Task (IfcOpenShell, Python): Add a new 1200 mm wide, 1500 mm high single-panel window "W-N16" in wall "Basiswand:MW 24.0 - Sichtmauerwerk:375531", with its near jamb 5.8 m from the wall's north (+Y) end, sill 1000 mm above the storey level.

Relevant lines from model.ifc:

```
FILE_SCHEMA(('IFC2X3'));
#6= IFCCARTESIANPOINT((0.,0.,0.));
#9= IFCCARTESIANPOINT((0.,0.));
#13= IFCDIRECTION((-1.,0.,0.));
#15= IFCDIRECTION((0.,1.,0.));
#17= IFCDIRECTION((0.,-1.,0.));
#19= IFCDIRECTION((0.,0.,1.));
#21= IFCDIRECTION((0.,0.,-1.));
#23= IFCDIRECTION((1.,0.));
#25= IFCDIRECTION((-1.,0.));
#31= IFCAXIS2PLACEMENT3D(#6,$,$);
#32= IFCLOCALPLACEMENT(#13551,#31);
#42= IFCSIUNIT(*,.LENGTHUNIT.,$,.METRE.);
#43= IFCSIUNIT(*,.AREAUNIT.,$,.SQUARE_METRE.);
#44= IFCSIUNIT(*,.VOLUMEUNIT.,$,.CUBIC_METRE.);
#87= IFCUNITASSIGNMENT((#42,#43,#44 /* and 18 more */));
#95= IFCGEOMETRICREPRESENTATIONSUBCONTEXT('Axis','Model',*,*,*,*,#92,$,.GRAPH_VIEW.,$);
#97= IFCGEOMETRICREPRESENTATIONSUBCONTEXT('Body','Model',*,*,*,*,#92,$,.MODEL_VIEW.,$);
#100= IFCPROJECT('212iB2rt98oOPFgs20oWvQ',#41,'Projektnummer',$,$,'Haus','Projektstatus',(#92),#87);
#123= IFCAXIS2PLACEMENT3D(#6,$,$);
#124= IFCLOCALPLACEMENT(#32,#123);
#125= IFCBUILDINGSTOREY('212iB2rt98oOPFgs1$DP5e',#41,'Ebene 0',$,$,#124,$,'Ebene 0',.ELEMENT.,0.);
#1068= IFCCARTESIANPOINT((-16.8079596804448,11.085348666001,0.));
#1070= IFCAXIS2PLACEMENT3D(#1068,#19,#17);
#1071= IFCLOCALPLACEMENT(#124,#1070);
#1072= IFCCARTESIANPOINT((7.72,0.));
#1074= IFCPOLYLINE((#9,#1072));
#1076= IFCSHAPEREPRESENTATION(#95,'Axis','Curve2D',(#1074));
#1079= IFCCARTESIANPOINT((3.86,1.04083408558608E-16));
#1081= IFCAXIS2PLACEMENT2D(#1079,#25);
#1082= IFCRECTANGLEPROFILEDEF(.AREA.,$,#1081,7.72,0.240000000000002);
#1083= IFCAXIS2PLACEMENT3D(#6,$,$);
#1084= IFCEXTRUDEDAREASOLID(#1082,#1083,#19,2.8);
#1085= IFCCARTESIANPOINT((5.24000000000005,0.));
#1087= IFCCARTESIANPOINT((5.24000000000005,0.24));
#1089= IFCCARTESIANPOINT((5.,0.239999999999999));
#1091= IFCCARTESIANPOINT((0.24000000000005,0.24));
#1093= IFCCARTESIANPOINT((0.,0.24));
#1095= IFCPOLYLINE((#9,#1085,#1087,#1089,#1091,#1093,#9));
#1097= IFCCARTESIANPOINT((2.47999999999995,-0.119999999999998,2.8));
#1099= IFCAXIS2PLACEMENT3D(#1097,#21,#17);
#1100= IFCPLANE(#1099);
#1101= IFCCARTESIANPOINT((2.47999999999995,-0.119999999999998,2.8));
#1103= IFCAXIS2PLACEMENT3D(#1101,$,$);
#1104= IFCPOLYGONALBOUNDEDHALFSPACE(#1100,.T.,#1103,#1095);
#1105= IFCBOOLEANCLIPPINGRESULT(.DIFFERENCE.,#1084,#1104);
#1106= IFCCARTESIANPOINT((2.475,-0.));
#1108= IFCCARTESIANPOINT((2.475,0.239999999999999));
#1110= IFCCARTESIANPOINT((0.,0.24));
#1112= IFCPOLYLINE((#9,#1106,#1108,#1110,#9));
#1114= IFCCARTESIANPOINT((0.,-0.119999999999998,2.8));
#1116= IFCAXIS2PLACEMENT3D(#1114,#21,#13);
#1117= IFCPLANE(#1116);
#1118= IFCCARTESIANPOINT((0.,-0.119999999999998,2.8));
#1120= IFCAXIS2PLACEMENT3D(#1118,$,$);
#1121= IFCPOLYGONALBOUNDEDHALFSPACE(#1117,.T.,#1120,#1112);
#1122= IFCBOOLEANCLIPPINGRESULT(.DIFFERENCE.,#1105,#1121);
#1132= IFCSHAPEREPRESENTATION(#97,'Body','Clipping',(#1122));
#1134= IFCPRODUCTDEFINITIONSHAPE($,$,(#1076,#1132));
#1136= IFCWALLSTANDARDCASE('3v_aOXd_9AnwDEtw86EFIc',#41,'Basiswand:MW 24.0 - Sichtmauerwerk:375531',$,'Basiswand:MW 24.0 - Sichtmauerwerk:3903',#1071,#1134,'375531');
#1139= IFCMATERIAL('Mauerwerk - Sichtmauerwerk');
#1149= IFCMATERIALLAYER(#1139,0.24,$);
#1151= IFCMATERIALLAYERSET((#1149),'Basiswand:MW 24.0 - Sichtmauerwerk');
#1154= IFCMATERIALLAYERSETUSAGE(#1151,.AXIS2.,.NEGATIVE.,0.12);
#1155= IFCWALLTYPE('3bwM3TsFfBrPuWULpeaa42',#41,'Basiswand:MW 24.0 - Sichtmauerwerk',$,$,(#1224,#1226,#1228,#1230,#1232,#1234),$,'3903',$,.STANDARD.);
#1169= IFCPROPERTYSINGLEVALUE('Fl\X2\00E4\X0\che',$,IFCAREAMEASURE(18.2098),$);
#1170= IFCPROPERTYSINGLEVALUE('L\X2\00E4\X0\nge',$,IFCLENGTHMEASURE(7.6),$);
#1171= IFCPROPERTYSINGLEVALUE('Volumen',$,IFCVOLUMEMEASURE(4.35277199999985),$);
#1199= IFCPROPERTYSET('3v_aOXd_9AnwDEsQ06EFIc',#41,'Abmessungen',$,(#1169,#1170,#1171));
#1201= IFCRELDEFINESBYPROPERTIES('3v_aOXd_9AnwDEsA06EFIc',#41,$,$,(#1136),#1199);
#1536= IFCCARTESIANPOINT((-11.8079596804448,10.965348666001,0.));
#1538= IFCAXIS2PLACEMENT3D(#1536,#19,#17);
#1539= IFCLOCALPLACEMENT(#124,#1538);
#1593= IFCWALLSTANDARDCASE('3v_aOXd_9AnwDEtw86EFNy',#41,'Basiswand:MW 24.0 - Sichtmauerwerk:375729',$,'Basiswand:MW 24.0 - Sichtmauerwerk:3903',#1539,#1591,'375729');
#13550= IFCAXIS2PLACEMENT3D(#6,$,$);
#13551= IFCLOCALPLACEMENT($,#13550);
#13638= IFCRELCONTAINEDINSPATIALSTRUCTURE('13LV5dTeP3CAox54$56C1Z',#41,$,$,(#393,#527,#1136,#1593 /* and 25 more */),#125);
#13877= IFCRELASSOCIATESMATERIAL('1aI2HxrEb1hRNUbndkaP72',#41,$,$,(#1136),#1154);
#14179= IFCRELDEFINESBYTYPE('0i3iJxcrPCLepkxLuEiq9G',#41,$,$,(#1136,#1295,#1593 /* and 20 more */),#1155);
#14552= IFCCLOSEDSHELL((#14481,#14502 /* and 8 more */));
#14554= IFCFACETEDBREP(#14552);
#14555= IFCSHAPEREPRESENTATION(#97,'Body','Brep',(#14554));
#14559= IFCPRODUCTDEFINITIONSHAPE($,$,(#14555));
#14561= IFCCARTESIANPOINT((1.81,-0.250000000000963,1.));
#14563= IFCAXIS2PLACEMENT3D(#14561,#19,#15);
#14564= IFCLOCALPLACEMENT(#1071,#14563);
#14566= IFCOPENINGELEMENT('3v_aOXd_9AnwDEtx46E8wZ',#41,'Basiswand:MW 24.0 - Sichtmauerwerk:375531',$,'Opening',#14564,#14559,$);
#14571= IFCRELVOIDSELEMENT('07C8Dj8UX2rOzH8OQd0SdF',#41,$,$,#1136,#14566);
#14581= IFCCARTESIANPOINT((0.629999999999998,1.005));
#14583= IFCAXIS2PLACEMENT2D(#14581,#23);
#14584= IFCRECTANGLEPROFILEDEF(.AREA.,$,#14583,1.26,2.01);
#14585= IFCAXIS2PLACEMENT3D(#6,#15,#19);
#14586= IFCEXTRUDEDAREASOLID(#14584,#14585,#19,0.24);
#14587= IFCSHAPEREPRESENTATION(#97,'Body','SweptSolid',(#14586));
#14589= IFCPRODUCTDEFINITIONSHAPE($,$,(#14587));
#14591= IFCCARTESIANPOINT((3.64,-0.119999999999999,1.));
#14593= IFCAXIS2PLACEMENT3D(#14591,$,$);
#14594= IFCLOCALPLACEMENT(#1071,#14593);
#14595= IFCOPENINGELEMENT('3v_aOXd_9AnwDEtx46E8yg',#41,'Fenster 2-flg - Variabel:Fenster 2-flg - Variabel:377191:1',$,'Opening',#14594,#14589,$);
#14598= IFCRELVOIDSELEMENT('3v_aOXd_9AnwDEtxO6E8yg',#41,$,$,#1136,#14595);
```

```python
import numpy as np
import ifcopenshell
import ifcopenshell.api.feature
import ifcopenshell.api.geometry
import ifcopenshell.api.pset
import ifcopenshell.api.root
import ifcopenshell.api.spatial
import ifcopenshell.api.type
import ifcopenshell.geom
import ifcopenshell.util.element
import ifcopenshell.util.placement
import ifcopenshell.util.representation
import ifcopenshell.util.shape
import ifcopenshell.util.unit

model = ifcopenshell.open("model.ifc")
unit_scale = ifcopenshell.util.unit.calculate_unit_scale(model)
area_scale = ifcopenshell.util.unit.calculate_unit_scale(model, "AREAUNIT")
volume_scale = ifcopenshell.util.unit.calculate_unit_scale(model, "VOLUMEUNIT")
settings = ifcopenshell.geom.settings()


def volume(element):
    """Net volume in cubic metres, openings subtracted."""
    shape = ifcopenshell.geom.create_shape(settings, element)
    return ifcopenshell.util.shape.get_volume(shape.geometry)


wall = model.by_guid("3v_aOXd_9AnwDEtw86EFIc")
storey = ifcopenshell.util.element.get_container(wall, ifc_class="IfcBuildingStorey")
context = ifcopenshell.util.representation.get_context(model, "Model", "Body", "MODEL_VIEW")
before = volume(wall)

width, height, from_end, sill = 1.2, 1.5, 5.8, 1  # metres

# The wall runs along its own X axis, and the end named is its -X end.
wall_shape = ifcopenshell.geom.create_shape(settings, wall)
x, y, z = ifcopenshell.util.shape.get_vertices(wall_shape.geometry).T
start = x.min() + from_end
face, thickness = float(y.min()), float(y.max() - y.min())
wall_matrix = ifcopenshell.util.placement.get_local_placement(wall.ObjectPlacement)
level = ifcopenshell.util.placement.get_local_placement(storey.ObjectPlacement)[2, 3]


def in_wall(x, y):
    """Placement at x, y metres in the wall's axes, at sill height."""
    matrix = wall_matrix.copy()
    matrix[:, 3] = wall_matrix @ np.array([x / unit_scale, y / unit_scale, 0.0, 1.0])
    matrix[2, 3] = level + sill / unit_scale
    return matrix


# Opening: a box that overshoots both wall faces by 50 mm.
opening = ifcopenshell.api.root.create_entity(model, ifc_class="IfcOpeningElement")
box = ifcopenshell.api.geometry.add_wall_representation(
    model, context=context, length=width, height=height, thickness=thickness + 0.1
)
ifcopenshell.api.geometry.assign_representation(model, product=opening, representation=box)
ifcopenshell.api.geometry.edit_object_placement(model, product=opening, matrix=in_wall(start, face - 0.05), is_si=False)
ifcopenshell.api.feature.add_feature(model, feature=opening, element=wall)

window = ifcopenshell.api.root.create_entity(model, ifc_class="IfcWindow", name="W-N16")
window.OverallWidth, window.OverallHeight = width / unit_scale, height / unit_scale
body = ifcopenshell.api.geometry.add_window_representation(
    model,
    context=context,
    overall_width=window.OverallWidth,
    overall_height=window.OverallHeight,
    partition_type="SINGLE_PANEL",
)
ifcopenshell.api.geometry.assign_representation(model, product=window, representation=body)
ifcopenshell.api.spatial.assign_container(model, products=[window], relating_structure=storey)
fills = ifcopenshell.api.feature.add_filling(model, opening=opening, element=window)
fills.OwnerHistory = window.OwnerHistory  # required in IFC2X3

# IFC2X3 keeps the operation on the window style.
style = ifcopenshell.api.root.create_entity(model, ifc_class="IfcWindowStyle", name="W-N16")
style.OperationType, style.ConstructionType = "SINGLE_PANEL", "NOTDEFINED"
style.ParameterTakesPrecedence = style.Sizeable = False
ifcopenshell.api.type.assign_type(model, related_objects=[window], relating_type=style)

# Centre the window in the wall's thickness.
ifcopenshell.api.geometry.edit_object_placement(model, product=window, matrix=in_wall(start, face), is_si=False)
window_shape = ifcopenshell.geom.create_shape(settings, window)
depth = ifcopenshell.util.shape.get_vertices(window_shape.geometry)[:, 1]
offset = face + thickness / 2 - (depth.min() + depth.max()) / 2
ifcopenshell.api.geometry.edit_object_placement(model, product=window, matrix=in_wall(start, offset), is_si=False)

after = volume(wall)

# Update the wall's stored quantities.
pset = model.by_id(ifcopenshell.util.element.get_pset(wall, "Abmessungen", should_inherit=False)["id"])
ifcopenshell.api.pset.edit_pset(model, pset=pset, properties={
    "Fläche": model.create_entity("IfcAreaMeasure", after / thickness / area_scale),
    "Volumen": model.create_entity("IfcVolumeMeasure", after / volume_scale),
})

print(f"wall volume {before:.3f} -> {after:.3f} m3")

model.write("model_edited.ifc")
```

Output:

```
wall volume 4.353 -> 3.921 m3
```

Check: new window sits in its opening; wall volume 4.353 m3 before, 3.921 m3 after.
